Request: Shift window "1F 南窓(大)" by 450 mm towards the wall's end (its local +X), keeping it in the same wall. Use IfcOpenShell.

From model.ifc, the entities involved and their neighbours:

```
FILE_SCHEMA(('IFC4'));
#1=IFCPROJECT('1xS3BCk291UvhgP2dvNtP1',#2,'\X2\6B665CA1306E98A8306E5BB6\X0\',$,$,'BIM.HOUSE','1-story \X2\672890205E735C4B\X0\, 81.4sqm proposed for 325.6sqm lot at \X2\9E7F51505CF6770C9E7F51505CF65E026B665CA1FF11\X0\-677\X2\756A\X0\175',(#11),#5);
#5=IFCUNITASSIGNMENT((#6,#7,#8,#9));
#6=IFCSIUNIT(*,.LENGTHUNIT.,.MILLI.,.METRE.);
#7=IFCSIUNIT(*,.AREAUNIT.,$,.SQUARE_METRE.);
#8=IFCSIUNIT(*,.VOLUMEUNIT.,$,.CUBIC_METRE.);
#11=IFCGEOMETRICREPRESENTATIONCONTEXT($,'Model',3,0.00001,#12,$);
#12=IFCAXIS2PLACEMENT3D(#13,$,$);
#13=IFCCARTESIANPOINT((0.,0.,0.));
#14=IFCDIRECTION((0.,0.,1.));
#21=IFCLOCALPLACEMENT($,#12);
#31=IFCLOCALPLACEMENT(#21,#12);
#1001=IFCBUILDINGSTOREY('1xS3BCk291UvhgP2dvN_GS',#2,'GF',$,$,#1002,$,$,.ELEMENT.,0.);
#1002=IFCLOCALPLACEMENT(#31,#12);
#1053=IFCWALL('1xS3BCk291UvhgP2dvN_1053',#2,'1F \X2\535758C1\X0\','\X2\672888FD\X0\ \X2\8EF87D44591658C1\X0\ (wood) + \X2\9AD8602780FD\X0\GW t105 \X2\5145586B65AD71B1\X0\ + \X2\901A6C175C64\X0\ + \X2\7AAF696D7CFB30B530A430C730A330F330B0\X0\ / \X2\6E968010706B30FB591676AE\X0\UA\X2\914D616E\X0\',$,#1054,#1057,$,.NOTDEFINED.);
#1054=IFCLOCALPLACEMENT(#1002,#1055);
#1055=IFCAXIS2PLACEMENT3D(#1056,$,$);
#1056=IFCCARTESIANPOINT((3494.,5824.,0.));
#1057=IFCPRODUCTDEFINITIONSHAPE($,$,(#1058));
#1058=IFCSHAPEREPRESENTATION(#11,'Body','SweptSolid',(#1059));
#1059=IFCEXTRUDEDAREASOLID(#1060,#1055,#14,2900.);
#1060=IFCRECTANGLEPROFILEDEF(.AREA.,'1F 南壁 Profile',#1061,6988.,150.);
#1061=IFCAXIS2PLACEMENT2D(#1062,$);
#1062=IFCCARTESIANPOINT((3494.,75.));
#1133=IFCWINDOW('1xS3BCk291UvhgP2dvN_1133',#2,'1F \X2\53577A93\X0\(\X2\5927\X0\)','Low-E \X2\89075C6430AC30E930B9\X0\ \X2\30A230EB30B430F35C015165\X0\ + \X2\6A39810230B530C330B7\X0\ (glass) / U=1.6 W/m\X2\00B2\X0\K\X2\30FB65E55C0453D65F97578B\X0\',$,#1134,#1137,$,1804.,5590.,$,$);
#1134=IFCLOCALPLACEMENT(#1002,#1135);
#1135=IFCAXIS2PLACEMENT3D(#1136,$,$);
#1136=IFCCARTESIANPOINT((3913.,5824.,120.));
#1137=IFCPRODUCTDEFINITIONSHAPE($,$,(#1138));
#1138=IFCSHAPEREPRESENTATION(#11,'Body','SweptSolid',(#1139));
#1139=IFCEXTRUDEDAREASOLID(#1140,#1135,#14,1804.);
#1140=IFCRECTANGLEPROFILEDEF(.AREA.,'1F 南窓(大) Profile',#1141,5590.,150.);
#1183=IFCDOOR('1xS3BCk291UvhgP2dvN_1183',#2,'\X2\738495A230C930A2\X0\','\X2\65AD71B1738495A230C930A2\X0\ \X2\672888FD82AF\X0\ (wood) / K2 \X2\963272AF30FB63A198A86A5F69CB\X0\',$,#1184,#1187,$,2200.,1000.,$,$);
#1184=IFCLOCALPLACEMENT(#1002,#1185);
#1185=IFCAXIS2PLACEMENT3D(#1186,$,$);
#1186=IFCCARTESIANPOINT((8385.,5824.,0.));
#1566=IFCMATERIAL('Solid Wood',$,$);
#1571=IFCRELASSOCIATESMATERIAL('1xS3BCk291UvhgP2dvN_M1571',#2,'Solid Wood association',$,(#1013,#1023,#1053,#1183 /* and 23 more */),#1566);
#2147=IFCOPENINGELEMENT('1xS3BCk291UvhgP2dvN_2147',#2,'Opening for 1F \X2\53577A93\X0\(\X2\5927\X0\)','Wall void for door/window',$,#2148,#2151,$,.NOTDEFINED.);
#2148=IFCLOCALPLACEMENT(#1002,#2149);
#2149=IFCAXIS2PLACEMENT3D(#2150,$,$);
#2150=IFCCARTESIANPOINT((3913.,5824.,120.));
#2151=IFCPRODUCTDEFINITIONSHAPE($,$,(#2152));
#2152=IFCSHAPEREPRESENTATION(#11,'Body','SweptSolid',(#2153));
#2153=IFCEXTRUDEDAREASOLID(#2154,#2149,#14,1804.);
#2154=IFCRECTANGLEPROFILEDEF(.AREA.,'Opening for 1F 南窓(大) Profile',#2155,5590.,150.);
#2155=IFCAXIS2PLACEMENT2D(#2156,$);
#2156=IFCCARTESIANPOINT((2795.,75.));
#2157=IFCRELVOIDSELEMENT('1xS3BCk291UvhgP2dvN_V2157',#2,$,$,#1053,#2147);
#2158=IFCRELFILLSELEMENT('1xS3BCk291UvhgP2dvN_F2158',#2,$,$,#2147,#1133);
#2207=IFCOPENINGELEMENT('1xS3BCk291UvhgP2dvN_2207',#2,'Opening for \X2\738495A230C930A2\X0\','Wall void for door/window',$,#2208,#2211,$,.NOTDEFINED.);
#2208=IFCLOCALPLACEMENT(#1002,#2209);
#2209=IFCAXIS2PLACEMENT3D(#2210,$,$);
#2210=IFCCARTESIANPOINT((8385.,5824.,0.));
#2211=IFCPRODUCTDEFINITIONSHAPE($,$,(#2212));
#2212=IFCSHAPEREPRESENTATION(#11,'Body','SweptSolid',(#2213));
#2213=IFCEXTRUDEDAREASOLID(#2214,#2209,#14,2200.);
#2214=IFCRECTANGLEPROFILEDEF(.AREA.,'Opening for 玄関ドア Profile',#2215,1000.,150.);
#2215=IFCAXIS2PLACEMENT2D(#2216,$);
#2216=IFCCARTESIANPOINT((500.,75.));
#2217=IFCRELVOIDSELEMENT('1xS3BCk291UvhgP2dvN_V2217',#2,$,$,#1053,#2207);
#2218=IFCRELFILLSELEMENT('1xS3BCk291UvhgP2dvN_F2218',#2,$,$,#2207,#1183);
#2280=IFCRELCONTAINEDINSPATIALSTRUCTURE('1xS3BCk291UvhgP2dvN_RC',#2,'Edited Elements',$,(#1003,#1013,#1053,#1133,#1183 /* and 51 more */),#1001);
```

```python
import ifcopenshell
import ifcopenshell.api.geometry
import ifcopenshell.util.placement
import ifcopenshell.util.unit

model = ifcopenshell.open("model.ifc")
unit_scale = ifcopenshell.util.unit.calculate_unit_scale(model)

window = model.by_guid("1xS3BCk291UvhgP2dvN_1133")
opening = window.FillsVoids[0].RelatingOpeningElement
wall = opening.VoidsElements[0].RelatingBuildingElement

wall_matrix = ifcopenshell.util.placement.get_local_placement(wall.ObjectPlacement)
shift = wall_matrix[:3, 0] * 0.45 / unit_scale
before = ifcopenshell.util.placement.get_local_placement(window.ObjectPlacement)[:3, 3].copy()

# The window is not placed relative to its opening, so move both.
for product in (opening, window):
    matrix = ifcopenshell.util.placement.get_local_placement(product.ObjectPlacement)
    matrix[:3, 3] += shift
    ifcopenshell.api.geometry.edit_object_placement(model, product=product, matrix=matrix, is_si=False)

after = ifcopenshell.util.placement.get_local_placement(window.ObjectPlacement)[:3, 3]
print("window moved by", (after - before).round(3) + 0.0)

model.write("model-out.ifc")
```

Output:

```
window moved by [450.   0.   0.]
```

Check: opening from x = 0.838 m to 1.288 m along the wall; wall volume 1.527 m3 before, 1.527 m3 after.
